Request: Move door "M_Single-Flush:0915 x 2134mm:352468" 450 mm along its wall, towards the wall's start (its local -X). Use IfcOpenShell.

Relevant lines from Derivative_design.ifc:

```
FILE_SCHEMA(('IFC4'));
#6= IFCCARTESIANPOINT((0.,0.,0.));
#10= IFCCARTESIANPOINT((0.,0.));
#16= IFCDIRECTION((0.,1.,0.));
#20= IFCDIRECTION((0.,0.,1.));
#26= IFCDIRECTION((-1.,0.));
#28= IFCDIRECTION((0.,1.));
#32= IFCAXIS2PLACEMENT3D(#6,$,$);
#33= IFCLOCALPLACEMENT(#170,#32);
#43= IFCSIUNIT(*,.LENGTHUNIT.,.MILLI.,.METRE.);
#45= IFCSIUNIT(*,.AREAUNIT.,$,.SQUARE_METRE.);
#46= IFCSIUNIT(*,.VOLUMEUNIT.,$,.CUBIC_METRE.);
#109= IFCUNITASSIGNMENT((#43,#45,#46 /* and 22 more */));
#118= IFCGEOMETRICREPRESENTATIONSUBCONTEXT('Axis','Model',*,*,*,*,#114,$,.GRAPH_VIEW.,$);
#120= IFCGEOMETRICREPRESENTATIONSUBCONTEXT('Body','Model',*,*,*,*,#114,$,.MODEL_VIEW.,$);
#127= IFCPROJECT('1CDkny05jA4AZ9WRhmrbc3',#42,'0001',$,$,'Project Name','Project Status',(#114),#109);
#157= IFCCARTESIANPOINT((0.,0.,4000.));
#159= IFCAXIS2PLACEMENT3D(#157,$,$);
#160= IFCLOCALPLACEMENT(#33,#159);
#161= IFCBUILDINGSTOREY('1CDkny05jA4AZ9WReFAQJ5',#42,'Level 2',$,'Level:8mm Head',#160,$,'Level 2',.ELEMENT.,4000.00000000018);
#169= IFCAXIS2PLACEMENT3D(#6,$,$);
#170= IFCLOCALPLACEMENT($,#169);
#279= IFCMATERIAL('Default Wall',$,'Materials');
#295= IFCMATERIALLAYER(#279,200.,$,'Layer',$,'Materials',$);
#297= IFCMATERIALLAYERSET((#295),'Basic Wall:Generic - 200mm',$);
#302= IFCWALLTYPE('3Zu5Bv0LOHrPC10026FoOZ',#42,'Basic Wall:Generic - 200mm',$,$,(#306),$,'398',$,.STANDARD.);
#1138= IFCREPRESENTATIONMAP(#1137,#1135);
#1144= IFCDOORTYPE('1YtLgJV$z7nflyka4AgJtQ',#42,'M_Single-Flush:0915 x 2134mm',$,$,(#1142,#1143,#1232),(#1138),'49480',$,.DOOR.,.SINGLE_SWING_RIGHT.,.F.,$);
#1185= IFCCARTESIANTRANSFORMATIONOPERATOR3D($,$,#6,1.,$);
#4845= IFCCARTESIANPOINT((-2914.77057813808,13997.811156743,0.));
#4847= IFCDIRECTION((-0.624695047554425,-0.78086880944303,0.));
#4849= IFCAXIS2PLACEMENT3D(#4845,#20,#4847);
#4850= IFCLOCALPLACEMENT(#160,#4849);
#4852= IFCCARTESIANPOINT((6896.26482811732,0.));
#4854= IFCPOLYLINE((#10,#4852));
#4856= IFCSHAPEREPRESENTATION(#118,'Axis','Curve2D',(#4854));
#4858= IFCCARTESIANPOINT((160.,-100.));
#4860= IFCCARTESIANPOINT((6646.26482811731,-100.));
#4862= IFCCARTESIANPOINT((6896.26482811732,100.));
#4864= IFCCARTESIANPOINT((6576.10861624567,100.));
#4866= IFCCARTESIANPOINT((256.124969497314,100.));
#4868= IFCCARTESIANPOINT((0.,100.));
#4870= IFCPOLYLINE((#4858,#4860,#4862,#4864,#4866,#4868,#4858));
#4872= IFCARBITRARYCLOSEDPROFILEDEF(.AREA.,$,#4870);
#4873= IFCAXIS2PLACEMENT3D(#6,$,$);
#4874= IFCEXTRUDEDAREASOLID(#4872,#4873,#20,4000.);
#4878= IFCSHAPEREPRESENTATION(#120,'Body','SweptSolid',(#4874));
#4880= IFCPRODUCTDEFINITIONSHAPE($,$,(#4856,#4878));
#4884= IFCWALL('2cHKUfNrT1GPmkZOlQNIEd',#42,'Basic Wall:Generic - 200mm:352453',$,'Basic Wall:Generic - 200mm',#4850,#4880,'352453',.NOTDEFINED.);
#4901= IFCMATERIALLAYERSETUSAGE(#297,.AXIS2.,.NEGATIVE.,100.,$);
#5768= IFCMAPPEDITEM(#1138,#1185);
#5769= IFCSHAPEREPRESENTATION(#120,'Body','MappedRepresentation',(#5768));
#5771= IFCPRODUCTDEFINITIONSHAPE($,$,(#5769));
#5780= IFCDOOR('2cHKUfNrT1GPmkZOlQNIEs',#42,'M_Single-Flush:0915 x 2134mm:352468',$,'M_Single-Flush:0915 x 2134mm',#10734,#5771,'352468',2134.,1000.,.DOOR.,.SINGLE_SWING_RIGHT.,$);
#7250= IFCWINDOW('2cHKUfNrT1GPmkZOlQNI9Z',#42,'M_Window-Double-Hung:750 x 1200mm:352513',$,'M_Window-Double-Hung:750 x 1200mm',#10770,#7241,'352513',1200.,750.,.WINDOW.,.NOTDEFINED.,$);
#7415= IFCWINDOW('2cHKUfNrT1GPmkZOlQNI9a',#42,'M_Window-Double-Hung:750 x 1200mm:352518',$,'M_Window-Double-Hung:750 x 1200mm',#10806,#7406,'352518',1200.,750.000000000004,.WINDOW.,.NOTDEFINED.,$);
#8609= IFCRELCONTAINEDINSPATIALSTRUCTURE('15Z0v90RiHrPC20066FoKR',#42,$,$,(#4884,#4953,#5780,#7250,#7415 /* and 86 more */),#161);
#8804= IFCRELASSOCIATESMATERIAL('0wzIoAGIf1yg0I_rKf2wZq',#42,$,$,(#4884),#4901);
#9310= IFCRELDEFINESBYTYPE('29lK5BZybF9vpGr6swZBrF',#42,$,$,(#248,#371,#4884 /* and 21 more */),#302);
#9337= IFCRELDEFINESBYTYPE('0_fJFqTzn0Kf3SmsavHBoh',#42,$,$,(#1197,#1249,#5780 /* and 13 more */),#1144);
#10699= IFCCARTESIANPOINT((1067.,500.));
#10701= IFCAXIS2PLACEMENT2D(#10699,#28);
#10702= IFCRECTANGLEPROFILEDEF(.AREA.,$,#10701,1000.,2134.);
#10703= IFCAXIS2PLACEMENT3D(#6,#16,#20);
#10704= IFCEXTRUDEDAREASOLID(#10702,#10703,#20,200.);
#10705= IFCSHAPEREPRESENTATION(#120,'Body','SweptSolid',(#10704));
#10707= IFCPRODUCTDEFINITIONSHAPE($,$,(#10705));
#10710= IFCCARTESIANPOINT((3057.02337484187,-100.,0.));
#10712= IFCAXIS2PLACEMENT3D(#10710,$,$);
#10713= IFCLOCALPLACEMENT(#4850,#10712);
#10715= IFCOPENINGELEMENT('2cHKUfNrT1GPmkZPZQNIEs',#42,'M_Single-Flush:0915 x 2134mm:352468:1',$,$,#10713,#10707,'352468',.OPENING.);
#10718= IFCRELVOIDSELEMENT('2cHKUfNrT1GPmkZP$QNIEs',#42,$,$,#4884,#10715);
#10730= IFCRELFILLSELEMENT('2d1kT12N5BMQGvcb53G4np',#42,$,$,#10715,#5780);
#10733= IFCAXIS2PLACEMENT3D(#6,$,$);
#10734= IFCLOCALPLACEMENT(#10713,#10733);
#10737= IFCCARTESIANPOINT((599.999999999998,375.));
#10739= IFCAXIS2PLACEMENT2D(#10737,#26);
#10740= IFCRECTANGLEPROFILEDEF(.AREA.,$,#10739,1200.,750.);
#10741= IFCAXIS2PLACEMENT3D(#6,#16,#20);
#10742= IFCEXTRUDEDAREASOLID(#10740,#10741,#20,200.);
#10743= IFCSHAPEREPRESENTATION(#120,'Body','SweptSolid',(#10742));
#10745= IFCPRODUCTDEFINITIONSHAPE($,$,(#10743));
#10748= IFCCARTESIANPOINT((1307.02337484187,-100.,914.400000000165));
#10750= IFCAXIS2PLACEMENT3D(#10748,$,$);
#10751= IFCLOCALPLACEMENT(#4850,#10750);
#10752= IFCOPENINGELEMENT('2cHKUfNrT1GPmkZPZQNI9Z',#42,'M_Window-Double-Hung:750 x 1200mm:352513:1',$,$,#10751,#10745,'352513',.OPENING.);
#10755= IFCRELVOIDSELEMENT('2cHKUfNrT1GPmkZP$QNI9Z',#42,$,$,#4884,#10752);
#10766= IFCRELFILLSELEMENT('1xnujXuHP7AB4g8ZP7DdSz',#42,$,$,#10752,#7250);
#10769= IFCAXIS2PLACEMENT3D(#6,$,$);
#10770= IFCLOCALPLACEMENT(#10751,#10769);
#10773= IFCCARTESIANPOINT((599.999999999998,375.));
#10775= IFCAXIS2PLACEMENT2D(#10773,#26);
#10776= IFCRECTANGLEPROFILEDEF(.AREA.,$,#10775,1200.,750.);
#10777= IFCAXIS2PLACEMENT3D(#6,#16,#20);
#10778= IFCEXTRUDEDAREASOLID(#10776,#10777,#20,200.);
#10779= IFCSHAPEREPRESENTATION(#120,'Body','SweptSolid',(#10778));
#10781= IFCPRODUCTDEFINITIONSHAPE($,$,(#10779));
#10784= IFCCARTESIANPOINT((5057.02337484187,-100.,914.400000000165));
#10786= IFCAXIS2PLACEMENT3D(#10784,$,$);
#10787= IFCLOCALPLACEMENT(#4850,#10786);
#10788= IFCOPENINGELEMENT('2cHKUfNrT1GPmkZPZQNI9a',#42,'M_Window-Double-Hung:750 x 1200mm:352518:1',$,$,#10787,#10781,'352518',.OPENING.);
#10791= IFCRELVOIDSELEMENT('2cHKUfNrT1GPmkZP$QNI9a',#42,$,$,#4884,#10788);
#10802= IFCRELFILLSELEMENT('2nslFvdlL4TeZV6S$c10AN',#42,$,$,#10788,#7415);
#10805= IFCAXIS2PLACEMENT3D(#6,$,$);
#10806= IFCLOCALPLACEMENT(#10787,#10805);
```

```python
import ifcopenshell
import ifcopenshell.api.geometry
import ifcopenshell.util.placement

model = ifcopenshell.open("Derivative_design.ifc")

door = model.by_id(5780)
opening = door.FillsVoids[0].RelatingOpeningElement
wall = opening.VoidsElements[0].RelatingBuildingElement

wall_matrix = ifcopenshell.util.placement.get_local_placement(wall.ObjectPlacement)
shift = wall_matrix[:3, 0] * -450.0
before = ifcopenshell.util.placement.get_local_placement(door.ObjectPlacement)[:3, 3].copy()

# The door is placed relative to its opening, so it follows when the opening moves.
matrix = ifcopenshell.util.placement.get_local_placement(opening.ObjectPlacement)
matrix[:3, 3] += shift
ifcopenshell.api.geometry.edit_object_placement(
    model, product=opening, matrix=matrix, is_si=False, should_transform_children=True
)

after = ifcopenshell.util.placement.get_local_placement(door.ObjectPlacement)[:3, 3]
print("door moved by", (after - before).round(3) + 0.0)

model.write("Derivative_design_edited.ifc")
```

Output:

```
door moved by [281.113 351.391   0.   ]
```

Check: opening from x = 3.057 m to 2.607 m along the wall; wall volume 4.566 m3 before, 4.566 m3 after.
